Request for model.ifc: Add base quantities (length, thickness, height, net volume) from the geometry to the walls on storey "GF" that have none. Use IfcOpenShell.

First a look at what the model holds.

```python
import ifcopenshell
import ifcopenshell.util.element
import ifcopenshell.util.unit

model = ifcopenshell.open("model.ifc")
print(model.schema)
for unit_type in ("LENGTHUNIT", "AREAUNIT", "VOLUMEUNIT"):
    print(unit_type, ifcopenshell.util.unit.calculate_unit_scale(model, unit_type))
storey = next(s for s in model.by_type("IfcBuildingStorey") if s.Name == "GF")
walls = [e for e in ifcopenshell.util.element.get_decomposition(storey) if e.is_a("IfcWall")]
for e in sorted(walls, key=lambda e: e.id()):
    print(e.id(), e.is_a(), e.Name, list(ifcopenshell.util.element.get_psets(e, qtos_only=True)), sep=" | ")
```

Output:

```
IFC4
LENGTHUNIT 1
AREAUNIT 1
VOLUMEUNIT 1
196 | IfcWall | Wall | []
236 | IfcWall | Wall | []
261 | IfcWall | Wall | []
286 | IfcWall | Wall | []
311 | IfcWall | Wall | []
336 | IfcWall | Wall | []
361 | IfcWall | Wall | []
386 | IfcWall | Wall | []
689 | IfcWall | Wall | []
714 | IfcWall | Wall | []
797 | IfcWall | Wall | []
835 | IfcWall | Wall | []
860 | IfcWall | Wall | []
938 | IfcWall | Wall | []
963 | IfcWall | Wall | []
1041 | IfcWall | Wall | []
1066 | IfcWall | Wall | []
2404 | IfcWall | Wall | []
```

```python
import ifcopenshell
import ifcopenshell.api.pset
import ifcopenshell.geom
import ifcopenshell.util.element
import ifcopenshell.util.shape
import ifcopenshell.util.unit

model = ifcopenshell.open("model.ifc")
unit_scale = ifcopenshell.util.unit.calculate_unit_scale(model)
volume_scale = ifcopenshell.util.unit.calculate_unit_scale(model, "VOLUMEUNIT")
settings = ifcopenshell.geom.settings()

storey = next(s for s in model.by_type("IfcBuildingStorey") if s.Name == "GF")
walls = [e for e in ifcopenshell.util.element.get_decomposition(storey) if e.is_a("IfcWall")]

for e in sorted(walls, key=lambda e: e.id()):
    if ifcopenshell.util.element.get_psets(e, qtos_only=True, should_inherit=False):
        continue
    # Geometry comes back in metres, in the element's own axes.
    shape = ifcopenshell.geom.create_shape(settings, e)
    values = {
        "Length": ifcopenshell.util.shape.get_x(shape.geometry) / unit_scale,
        "Width": ifcopenshell.util.shape.get_y(shape.geometry) / unit_scale,
        "Height": ifcopenshell.util.shape.get_z(shape.geometry) / unit_scale,
        "NetVolume": ifcopenshell.util.shape.get_volume(shape.geometry) / volume_scale,
    }
    qto = ifcopenshell.api.pset.add_qto(model, product=e, name="Qto_WallBaseQuantities")
    ifcopenshell.api.pset.edit_qto(model, qto=qto, properties=values)
    print(e.id(), {k: round(v, 3) for k, v in values.items()})

model.write("model_edited.ifc")
```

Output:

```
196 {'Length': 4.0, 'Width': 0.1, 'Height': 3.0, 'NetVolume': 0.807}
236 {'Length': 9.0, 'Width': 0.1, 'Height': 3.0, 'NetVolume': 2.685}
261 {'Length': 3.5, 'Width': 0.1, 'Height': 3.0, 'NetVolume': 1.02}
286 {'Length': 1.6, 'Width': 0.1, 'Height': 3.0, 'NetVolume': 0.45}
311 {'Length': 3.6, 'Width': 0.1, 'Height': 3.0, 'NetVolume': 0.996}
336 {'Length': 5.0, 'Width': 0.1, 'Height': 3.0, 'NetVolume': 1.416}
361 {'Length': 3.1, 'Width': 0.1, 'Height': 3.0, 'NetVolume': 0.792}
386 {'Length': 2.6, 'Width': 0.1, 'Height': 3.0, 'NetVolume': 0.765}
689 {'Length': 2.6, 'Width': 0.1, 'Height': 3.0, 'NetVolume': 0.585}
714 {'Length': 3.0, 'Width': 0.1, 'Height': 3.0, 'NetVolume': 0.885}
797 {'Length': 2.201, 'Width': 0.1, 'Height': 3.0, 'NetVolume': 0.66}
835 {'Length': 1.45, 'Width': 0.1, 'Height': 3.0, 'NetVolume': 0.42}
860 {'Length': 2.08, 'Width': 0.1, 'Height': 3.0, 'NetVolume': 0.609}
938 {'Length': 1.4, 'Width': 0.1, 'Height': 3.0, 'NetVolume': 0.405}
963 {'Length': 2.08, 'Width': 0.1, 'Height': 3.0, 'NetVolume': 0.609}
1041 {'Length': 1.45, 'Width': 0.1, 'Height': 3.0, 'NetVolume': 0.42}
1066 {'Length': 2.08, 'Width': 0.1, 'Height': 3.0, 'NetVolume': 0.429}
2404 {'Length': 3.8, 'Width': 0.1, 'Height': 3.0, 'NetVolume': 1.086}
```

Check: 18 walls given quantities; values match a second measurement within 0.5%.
